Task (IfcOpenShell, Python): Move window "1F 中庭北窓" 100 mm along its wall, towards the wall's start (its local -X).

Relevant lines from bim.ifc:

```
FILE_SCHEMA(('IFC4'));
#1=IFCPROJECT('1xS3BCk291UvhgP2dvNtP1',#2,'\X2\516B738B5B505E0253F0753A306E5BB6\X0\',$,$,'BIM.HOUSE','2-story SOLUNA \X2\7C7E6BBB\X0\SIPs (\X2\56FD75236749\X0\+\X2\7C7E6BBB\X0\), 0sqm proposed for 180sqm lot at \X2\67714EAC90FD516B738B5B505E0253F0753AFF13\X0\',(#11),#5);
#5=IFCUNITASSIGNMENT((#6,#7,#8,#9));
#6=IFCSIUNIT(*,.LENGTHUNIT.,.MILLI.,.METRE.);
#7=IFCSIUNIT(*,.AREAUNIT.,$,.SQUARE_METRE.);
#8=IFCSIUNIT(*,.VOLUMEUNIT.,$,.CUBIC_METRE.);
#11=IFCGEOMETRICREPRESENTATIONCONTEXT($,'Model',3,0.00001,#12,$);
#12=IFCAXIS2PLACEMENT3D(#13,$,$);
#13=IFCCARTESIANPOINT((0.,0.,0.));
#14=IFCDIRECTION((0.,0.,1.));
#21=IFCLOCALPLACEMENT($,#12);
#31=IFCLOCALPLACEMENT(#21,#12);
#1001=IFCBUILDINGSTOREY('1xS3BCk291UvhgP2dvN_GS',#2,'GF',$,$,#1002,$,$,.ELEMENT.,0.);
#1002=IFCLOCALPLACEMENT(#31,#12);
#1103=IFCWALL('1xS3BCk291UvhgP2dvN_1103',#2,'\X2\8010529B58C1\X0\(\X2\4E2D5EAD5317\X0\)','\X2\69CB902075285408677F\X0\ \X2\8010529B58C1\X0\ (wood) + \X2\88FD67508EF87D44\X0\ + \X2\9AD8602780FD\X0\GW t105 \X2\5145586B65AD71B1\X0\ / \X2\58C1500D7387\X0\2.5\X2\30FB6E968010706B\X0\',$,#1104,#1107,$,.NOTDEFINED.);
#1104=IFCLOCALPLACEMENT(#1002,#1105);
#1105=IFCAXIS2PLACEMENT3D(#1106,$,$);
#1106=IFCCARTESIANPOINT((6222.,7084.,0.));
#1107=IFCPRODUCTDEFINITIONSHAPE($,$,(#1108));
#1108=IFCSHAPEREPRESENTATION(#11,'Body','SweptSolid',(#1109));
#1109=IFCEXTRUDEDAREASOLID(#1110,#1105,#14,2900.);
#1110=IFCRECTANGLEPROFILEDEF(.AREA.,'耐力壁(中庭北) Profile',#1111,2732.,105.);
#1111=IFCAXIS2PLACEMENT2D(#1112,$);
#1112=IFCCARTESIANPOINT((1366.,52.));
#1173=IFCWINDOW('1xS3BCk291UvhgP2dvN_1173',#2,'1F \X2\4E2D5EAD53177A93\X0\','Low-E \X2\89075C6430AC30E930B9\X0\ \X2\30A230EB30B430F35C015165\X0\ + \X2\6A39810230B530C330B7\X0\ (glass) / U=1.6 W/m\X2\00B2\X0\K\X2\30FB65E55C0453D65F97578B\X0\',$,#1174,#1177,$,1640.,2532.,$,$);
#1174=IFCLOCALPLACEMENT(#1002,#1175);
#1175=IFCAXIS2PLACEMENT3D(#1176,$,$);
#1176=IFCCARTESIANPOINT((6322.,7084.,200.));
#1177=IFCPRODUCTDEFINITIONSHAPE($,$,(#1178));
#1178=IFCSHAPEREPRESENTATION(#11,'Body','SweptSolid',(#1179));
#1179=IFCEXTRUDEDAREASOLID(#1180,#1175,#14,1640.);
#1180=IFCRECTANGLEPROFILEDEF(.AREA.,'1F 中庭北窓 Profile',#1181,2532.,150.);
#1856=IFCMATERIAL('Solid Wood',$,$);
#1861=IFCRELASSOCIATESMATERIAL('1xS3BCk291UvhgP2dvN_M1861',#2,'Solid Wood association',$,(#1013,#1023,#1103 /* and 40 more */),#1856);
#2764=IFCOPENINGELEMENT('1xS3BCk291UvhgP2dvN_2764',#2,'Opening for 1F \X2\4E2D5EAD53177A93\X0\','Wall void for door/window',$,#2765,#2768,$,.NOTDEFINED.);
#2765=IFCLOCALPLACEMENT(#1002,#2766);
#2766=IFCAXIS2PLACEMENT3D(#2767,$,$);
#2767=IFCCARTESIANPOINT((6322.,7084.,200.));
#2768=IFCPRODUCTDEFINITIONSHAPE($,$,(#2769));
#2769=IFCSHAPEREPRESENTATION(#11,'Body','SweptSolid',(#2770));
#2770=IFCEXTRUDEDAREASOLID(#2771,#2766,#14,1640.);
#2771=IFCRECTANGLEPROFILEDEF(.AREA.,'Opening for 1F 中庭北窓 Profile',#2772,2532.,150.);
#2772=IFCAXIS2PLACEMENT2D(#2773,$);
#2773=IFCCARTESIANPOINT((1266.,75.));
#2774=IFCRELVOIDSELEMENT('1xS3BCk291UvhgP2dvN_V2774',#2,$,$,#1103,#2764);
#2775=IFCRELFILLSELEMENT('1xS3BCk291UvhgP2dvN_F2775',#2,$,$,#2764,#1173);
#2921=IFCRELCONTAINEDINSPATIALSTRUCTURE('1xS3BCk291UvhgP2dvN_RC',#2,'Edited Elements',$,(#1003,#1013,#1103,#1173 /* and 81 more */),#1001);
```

```python
import ifcopenshell
import ifcopenshell.api.geometry
import ifcopenshell.util.placement
import ifcopenshell.util.unit

model = ifcopenshell.open("bim.ifc")
unit_scale = ifcopenshell.util.unit.calculate_unit_scale(model)

window = model.by_guid("1xS3BCk291UvhgP2dvN_1173")
opening = window.FillsVoids[0].RelatingOpeningElement
wall = opening.VoidsElements[0].RelatingBuildingElement

wall_matrix = ifcopenshell.util.placement.get_local_placement(wall.ObjectPlacement)
shift = wall_matrix[:3, 0] * -0.1 / unit_scale
before = ifcopenshell.util.placement.get_local_placement(window.ObjectPlacement)[:3, 3].copy()

# The window is not placed relative to its opening, so move both.
for product in (opening, window):
    matrix = ifcopenshell.util.placement.get_local_placement(product.ObjectPlacement)
    matrix[:3, 3] += shift
    ifcopenshell.api.geometry.edit_object_placement(model, product=product, matrix=matrix, is_si=False)

after = ifcopenshell.util.placement.get_local_placement(window.ObjectPlacement)[:3, 3]
print("window moved by", (after - before).round(3) + 0.0)

model.write("bim_v2.ifc")
```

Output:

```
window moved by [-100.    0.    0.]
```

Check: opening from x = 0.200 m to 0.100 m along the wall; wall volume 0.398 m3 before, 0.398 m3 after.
